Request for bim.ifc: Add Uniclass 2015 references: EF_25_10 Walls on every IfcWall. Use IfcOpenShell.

First a look at what the model holds.

```python
import ifcopenshell

model = ifcopenshell.open("bim.ifc")
print(model.schema)
print("classifications:", [c.Name for c in model.by_type("IfcClassification")])
for ifc_class in ("IfcDoor", "IfcRoof", "IfcStair", "IfcWall", "IfcWindow"):
    print(ifc_class, len(model.by_type(ifc_class)))
```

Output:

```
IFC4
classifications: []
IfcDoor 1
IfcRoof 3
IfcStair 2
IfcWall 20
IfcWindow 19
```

```python
import ifcopenshell
import ifcopenshell.api.classification

model = ifcopenshell.open("bim.ifc")

system = ifcopenshell.api.classification.add_classification(model, classification="Uniclass 2015")

codes = {
    "IfcWall": ("EF_25_10", "Walls"),
}
for ifc_class, (code, name) in codes.items():
    products = model.by_type(ifc_class)
    ifcopenshell.api.classification.add_reference(
        model, products=products, classification=system, identification=code, name=name
    )
    print(code, len(products))

model.write("bim_v2.ifc")
```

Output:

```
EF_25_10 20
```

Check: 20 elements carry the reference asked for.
